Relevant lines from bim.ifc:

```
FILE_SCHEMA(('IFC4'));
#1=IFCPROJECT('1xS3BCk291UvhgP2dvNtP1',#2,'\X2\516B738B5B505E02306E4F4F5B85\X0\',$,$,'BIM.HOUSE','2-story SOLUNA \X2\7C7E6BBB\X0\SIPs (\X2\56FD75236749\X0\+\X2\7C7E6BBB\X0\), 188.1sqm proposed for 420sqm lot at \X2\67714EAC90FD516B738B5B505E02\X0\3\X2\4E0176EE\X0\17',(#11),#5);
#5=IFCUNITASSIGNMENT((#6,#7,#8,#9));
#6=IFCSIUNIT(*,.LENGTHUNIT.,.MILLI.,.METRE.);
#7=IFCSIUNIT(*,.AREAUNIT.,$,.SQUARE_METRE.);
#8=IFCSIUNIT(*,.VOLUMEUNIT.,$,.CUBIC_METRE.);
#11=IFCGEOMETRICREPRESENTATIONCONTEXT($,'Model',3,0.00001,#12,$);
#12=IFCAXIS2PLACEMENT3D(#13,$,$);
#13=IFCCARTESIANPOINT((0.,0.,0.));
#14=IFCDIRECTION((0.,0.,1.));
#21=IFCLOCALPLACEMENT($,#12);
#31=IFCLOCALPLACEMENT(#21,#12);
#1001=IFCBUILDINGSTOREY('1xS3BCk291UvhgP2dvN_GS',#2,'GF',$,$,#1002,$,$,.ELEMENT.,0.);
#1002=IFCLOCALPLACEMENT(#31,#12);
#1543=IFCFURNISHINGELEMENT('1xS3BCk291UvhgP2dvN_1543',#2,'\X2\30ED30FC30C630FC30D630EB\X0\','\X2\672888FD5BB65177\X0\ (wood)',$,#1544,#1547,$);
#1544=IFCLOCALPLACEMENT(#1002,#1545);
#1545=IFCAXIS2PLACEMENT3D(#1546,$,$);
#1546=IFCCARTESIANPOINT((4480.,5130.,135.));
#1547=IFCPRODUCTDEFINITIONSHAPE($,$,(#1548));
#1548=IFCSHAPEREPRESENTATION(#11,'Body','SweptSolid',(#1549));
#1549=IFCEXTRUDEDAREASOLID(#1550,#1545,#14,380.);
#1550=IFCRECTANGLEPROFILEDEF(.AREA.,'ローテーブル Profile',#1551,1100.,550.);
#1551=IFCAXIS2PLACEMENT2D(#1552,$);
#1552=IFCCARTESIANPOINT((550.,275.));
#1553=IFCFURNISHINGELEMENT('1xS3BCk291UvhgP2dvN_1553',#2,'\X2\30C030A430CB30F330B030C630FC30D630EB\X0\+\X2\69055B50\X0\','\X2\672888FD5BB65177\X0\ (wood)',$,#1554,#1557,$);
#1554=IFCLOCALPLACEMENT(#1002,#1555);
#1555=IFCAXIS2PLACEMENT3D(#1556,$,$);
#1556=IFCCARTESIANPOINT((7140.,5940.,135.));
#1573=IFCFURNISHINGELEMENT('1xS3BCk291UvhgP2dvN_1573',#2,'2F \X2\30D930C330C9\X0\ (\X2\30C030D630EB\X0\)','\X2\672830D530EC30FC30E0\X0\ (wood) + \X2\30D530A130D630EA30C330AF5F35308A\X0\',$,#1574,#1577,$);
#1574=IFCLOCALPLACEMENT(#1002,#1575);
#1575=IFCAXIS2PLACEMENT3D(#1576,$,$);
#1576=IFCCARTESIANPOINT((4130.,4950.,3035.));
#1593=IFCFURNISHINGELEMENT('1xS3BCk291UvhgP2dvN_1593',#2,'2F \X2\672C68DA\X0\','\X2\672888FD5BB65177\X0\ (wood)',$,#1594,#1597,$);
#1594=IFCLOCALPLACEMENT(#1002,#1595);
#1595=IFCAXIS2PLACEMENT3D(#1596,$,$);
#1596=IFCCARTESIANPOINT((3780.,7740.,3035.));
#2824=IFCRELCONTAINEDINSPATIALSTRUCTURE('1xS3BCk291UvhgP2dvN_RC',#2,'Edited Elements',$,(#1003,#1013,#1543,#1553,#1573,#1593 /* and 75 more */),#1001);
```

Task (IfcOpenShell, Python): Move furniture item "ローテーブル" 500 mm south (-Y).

```python
import ifcopenshell
import ifcopenshell.api.geometry
import ifcopenshell.util.placement

model = ifcopenshell.open("bim.ifc")

item = model.by_guid("1xS3BCk291UvhgP2dvN_1543")
matrix = ifcopenshell.util.placement.get_local_placement(item.ObjectPlacement)
matrix[1, 3] -= 500.0
ifcopenshell.api.geometry.edit_object_placement(model, product=item, matrix=matrix, is_si=False)

print(ifcopenshell.util.placement.get_local_placement(item.ObjectPlacement).round(3) + 0.0)

model.write("bim_edited.ifc")
```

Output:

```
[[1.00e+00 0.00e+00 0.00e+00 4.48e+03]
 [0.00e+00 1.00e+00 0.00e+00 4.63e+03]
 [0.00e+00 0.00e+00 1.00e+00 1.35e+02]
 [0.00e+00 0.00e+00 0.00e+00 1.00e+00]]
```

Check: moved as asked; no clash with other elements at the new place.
